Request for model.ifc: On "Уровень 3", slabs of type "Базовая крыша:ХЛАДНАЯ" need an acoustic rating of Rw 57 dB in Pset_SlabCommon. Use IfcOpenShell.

First a look at what the model holds.

```python
import ifcopenshell
import ifcopenshell.util.element

model = ifcopenshell.open("model.ifc")
print(model.schema)
storey = next(s for s in model.by_type("IfcBuildingStorey") if s.Name == "Уровень 3")
slabs = [e for e in ifcopenshell.util.element.get_decomposition(storey) if e.is_a("IfcSlab")]
seen = {}
for e in slabs:
    element_type = ifcopenshell.util.element.get_type(e)
    key = (element_type.Name if element_type != e and element_type else None, ifcopenshell.util.element.get_pset(e, "Pset_SlabCommon", "AcousticRating"))
    seen[key] = seen.get(key, 0) + 1
for (name, value), count in sorted(seen.items(), key=str):
    print(count, "x", name, "|", value)
```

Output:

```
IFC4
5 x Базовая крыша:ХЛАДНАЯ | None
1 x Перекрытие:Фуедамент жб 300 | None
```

```python
import ifcopenshell
import ifcopenshell.api.pset
import ifcopenshell.util.element

model = ifcopenshell.open("model.ifc")

storey = next(s for s in model.by_type("IfcBuildingStorey") if s.Name == "Уровень 3")
slabs = [e for e in ifcopenshell.util.element.get_decomposition(storey) if e.is_a("IfcSlab")]

count = 0
for e in slabs:
    element_type = ifcopenshell.util.element.get_type(e)
    if element_type in (None, e) or element_type.Name != "Базовая крыша:ХЛАДНАЯ":
        continue
    # add_pset returns the element's existing set when there is one.
    pset = ifcopenshell.api.pset.add_pset(model, product=e, name="Pset_SlabCommon")
    ifcopenshell.api.pset.edit_pset(model, pset=pset, properties={"AcousticRating": "Rw 57 dB"})
    count += 1

print(count, "slabs updated")

model.write("model_updated.ifc")
```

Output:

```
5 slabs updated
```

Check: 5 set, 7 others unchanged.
